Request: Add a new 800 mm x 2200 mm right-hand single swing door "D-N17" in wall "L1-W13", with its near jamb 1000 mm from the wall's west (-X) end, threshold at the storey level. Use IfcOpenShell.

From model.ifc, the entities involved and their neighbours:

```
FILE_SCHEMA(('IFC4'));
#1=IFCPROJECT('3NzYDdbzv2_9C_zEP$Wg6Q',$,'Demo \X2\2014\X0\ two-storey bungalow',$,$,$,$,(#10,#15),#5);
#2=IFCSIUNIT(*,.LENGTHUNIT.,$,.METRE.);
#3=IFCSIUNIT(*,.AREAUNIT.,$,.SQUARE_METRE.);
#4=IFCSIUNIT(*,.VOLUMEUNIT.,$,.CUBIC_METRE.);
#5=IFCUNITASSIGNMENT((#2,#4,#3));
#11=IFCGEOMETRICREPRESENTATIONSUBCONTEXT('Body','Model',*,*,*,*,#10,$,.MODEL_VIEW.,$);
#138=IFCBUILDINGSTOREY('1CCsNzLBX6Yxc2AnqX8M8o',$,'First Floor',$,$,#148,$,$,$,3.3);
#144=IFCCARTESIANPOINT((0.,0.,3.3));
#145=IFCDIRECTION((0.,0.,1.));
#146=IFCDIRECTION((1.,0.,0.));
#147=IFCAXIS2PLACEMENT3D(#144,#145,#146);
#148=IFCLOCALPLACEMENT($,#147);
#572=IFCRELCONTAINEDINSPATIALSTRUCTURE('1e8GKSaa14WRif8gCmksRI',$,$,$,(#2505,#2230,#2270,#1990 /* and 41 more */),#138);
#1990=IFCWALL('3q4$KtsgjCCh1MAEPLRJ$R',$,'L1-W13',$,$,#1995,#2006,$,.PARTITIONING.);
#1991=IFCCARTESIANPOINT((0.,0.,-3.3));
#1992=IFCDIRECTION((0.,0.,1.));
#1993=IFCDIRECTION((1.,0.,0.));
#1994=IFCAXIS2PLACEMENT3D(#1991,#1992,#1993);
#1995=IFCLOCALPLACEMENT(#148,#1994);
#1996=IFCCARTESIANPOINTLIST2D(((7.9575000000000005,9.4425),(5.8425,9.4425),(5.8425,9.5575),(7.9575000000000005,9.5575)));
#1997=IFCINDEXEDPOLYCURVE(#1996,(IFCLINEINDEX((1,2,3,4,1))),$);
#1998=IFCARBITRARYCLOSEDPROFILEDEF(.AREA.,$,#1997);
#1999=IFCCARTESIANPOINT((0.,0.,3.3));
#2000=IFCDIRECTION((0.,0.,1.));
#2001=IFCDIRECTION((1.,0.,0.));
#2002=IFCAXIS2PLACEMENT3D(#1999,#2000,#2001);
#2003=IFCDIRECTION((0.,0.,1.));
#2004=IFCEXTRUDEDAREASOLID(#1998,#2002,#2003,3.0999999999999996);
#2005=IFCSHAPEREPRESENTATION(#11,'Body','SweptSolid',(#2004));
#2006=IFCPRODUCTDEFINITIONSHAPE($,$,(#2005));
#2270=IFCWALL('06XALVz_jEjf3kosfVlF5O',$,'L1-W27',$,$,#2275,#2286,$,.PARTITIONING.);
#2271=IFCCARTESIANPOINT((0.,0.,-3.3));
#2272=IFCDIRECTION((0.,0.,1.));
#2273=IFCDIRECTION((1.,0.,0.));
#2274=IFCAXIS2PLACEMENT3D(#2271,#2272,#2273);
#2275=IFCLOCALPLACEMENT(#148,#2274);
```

```python
import numpy as np
import ifcopenshell
import ifcopenshell.api.feature
import ifcopenshell.api.geometry
import ifcopenshell.api.root
import ifcopenshell.api.spatial
import ifcopenshell.geom
import ifcopenshell.util.element
import ifcopenshell.util.placement
import ifcopenshell.util.representation
import ifcopenshell.util.shape
import ifcopenshell.util.unit

model = ifcopenshell.open("model.ifc")
unit_scale = ifcopenshell.util.unit.calculate_unit_scale(model)
settings = ifcopenshell.geom.settings()


def volume(element):
    """Net volume in cubic metres, openings subtracted."""
    shape = ifcopenshell.geom.create_shape(settings, element)
    return ifcopenshell.util.shape.get_volume(shape.geometry)


wall = model.by_guid("3q4$KtsgjCCh1MAEPLRJ$R")
storey = ifcopenshell.util.element.get_container(wall, ifc_class="IfcBuildingStorey")
context = ifcopenshell.util.representation.get_context(model, "Model", "Body", "MODEL_VIEW")
before = volume(wall)

width, height, from_end, sill = 0.8, 2.2, 1, 0.0  # metres

# The wall runs along its own X axis, and the end named is its -X end.
wall_shape = ifcopenshell.geom.create_shape(settings, wall)
x, y, z = ifcopenshell.util.shape.get_vertices(wall_shape.geometry).T
start = x.min() + from_end
face, thickness = float(y.min()), float(y.max() - y.min())
wall_matrix = ifcopenshell.util.placement.get_local_placement(wall.ObjectPlacement)
level = ifcopenshell.util.placement.get_local_placement(storey.ObjectPlacement)[2, 3]


def in_wall(x, y):
    """Placement at x, y metres in the wall's axes, at sill height."""
    matrix = wall_matrix.copy()
    matrix[:, 3] = wall_matrix @ np.array([x / unit_scale, y / unit_scale, 0.0, 1.0])
    matrix[2, 3] = level + sill / unit_scale
    return matrix


# Opening: a box that overshoots both wall faces by 50 mm.
opening = ifcopenshell.api.root.create_entity(model, ifc_class="IfcOpeningElement", predefined_type="OPENING")
box = ifcopenshell.api.geometry.add_wall_representation(
    model, context=context, length=width, height=height, thickness=thickness + 0.1
)
ifcopenshell.api.geometry.assign_representation(model, product=opening, representation=box)
ifcopenshell.api.geometry.edit_object_placement(model, product=opening, matrix=in_wall(start, face - 0.05), is_si=False)
ifcopenshell.api.feature.add_feature(model, feature=opening, element=wall)

door = ifcopenshell.api.root.create_entity(model, ifc_class="IfcDoor", name="D-N17", predefined_type="DOOR")
door.OverallWidth, door.OverallHeight = width / unit_scale, height / unit_scale
door.OperationType = "SINGLE_SWING_RIGHT"
body = ifcopenshell.api.geometry.add_door_representation(
    model,
    context=context,
    overall_width=door.OverallWidth,
    overall_height=door.OverallHeight,
    operation_type="SINGLE_SWING_RIGHT",
    lining_properties={"LiningDepth": thickness / unit_scale, "ThresholdDepth": thickness / unit_scale},
)
ifcopenshell.api.geometry.assign_representation(model, product=door, representation=body)
ifcopenshell.api.spatial.assign_container(model, products=[door], relating_structure=storey)
ifcopenshell.api.feature.add_filling(model, opening=opening, element=door)

# The lining spans the wall, so the door starts at the wall face.
ifcopenshell.api.geometry.edit_object_placement(model, product=door, matrix=in_wall(start, face), is_si=False)

after = volume(wall)

print(f"wall volume {before:.3f} -> {after:.3f} m3")

model.write("model_updated.ifc")
```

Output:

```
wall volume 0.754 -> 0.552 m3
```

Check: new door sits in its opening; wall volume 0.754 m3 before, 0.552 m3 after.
